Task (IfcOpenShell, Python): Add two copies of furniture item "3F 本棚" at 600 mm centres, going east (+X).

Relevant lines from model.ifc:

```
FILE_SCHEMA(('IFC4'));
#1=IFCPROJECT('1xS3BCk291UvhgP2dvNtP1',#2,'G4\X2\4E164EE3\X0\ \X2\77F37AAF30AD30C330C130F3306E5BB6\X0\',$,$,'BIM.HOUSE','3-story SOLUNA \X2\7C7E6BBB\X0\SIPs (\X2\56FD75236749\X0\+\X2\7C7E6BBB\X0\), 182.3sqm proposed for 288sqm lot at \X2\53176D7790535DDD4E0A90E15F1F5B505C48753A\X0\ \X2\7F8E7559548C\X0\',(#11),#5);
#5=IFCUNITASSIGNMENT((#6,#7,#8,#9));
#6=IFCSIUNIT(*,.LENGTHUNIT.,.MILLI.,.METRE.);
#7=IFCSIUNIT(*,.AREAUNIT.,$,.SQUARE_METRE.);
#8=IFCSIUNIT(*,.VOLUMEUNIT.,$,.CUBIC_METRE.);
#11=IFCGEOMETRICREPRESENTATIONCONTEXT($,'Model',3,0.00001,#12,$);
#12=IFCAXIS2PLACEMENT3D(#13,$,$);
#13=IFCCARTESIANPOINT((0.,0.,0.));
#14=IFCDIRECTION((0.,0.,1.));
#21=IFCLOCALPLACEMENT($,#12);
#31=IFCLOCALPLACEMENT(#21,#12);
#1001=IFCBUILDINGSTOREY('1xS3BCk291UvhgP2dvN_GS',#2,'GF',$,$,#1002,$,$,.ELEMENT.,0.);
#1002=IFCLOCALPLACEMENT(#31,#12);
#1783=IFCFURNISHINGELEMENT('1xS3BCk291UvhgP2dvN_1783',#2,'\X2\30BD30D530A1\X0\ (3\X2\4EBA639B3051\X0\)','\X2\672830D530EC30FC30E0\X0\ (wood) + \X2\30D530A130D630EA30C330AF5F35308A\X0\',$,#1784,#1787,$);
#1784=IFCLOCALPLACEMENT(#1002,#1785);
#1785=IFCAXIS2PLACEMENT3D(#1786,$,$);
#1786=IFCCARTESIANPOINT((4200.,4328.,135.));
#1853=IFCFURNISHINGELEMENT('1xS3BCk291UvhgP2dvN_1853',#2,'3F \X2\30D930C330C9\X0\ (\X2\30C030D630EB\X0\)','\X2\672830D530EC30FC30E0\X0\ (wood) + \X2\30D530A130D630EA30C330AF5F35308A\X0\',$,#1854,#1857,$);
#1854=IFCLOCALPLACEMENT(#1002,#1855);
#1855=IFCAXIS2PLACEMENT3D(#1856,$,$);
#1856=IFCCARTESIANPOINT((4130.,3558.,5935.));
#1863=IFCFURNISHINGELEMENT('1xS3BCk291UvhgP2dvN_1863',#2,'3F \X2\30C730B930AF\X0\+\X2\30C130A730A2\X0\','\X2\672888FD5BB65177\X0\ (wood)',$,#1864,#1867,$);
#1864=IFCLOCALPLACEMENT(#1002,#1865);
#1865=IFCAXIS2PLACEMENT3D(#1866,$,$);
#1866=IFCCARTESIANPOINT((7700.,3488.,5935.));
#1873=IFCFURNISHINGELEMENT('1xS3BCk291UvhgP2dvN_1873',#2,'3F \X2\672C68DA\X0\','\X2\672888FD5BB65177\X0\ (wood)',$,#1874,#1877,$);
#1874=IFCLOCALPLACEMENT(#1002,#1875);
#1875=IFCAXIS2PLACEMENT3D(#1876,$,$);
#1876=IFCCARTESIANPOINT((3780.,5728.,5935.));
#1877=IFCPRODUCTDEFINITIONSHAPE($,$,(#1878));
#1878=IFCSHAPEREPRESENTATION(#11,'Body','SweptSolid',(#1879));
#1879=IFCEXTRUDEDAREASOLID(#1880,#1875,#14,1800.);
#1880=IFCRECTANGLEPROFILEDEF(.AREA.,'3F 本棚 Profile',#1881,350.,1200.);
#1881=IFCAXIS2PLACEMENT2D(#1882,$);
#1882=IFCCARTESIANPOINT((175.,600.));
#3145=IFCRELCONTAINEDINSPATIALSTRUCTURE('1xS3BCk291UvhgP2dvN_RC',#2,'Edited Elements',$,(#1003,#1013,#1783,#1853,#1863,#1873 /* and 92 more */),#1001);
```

```python
import numpy as np
import ifcopenshell
import ifcopenshell.api.geometry
import ifcopenshell.api.root
import ifcopenshell.util.element
import ifcopenshell.util.placement

model = ifcopenshell.open("model.ifc")


def reuse_history(source, copy):
    """copy_class also copies each property set's owner history, people and application; keep the originals."""
    for rel in copy.IsDefinedBy:
        if rel.is_a("IfcRelDefinesByProperties") and (history := rel.RelatingPropertyDefinition.OwnerHistory):
            rel.RelatingPropertyDefinition.OwnerHistory = source.OwnerHistory
            ifcopenshell.util.element.remove_deep2(model, history)


source = model.by_id(1873)
base = ifcopenshell.util.placement.get_local_placement(source.ObjectPlacement)
step = np.array([1.0, 0.0, 0.0]) * 600.0

for i in range(1, 3):
    copy = ifcopenshell.api.root.copy_class(model, product=source)
    copy.Representation = ifcopenshell.util.element.copy_deep(
        model, source.Representation, exclude=["IfcGeometricRepresentationContext", "IfcRepresentationMap"]
    )
    reuse_history(source, copy)
    matrix = base.copy()
    matrix[:3, 3] += i * step
    print("added at", matrix[:3, 3].round(3) + 0.0)
    ifcopenshell.api.geometry.edit_object_placement(model, product=copy, matrix=matrix, is_si=False)

model.write("model_v2.ifc")
```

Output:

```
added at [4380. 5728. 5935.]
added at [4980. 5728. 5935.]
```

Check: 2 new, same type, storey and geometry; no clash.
